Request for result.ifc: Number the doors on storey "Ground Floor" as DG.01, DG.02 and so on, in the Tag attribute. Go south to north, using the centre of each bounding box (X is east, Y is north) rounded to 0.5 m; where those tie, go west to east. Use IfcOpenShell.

First a look at what the model holds.

```python
import ifcopenshell
import ifcopenshell.util.element
import ifcopenshell.util.placement

model = ifcopenshell.open("result.ifc")
print(model.schema)
storey = next(s for s in model.by_type("IfcBuildingStorey") if s.Name == "Ground Floor")
doors = [e for e in ifcopenshell.util.element.get_decomposition(storey) if e.is_a("IfcDoor")]
for e in sorted(doors, key=lambda e: e.id()):
    origin = ifcopenshell.util.placement.get_local_placement(e.ObjectPlacement)[:3, 3]
    print(e.id(), e.Tag, e.Name, origin.round(2) + 0.0, sep=" | ")
```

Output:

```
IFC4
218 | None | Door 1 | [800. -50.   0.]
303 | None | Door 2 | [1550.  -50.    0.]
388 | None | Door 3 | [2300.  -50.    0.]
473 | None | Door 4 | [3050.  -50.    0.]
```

```python
import ifcopenshell
import ifcopenshell.geom
import ifcopenshell.util.element
import ifcopenshell.util.shape

model = ifcopenshell.open("result.ifc")
settings = ifcopenshell.geom.settings()
settings.set("use-world-coords", True)


def centre(element):
    shape = ifcopenshell.geom.create_shape(settings, element)
    return ifcopenshell.util.shape.get_bbox_centroid(shape.geometry)


storey = next(s for s in model.by_type("IfcBuildingStorey") if s.Name == "Ground Floor")
doors = [e for e in ifcopenshell.util.element.get_decomposition(storey) if e.is_a("IfcDoor")]

# Insertion points can sit at a corner or the storey origin, so sort by the geometry (in metres).
centres = {e: centre(e) for e in doors}
doors.sort(key=lambda e: (round(centres[e][1] / 0.5), centres[e][0]))

for i, e in enumerate(doors, start=1):
    number = f"DG.{i:02d}"
    e.Tag = number
    print(e.id(), number)

model.write("result_updated.ifc")
```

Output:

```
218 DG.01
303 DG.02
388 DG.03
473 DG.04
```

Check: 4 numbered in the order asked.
